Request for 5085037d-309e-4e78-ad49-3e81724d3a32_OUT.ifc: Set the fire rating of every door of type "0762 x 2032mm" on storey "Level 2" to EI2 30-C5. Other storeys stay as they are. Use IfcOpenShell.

First a look at what the model holds.

```python
import ifcopenshell
import ifcopenshell.util.element

model = ifcopenshell.open("5085037d-309e-4e78-ad49-3e81724d3a32_OUT.ifc")
print(model.schema)
storey = next(s for s in model.by_type("IfcBuildingStorey") if s.Name == "Level 2")
doors = [e for e in ifcopenshell.util.element.get_decomposition(storey) if e.is_a("IfcDoor")]
seen = {}
for e in doors:
    element_type = ifcopenshell.util.element.get_type(e)
    key = (element_type.Name if element_type != e and element_type else None, ifcopenshell.util.element.get_pset(e, "Pset_DoorCommon", "FireRating"))
    seen[key] = seen.get(key, 0) + 1
for (name, value), count in sorted(seen.items(), key=str):
    print(count, "x", name, "|", value)
```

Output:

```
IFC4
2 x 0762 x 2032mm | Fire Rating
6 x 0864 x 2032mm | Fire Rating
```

```python
import ifcopenshell
import ifcopenshell.api.pset
import ifcopenshell.util.element

model = ifcopenshell.open("5085037d-309e-4e78-ad49-3e81724d3a32_OUT.ifc")

storey = next(s for s in model.by_type("IfcBuildingStorey") if s.Name == "Level 2")
doors = [e for e in ifcopenshell.util.element.get_decomposition(storey) if e.is_a("IfcDoor")]

count = 0
for e in doors:
    element_type = ifcopenshell.util.element.get_type(e)
    if element_type in (None, e) or element_type.Name != "0762 x 2032mm":
        continue
    # add_pset returns the element's existing set when there is one.
    pset = ifcopenshell.api.pset.add_pset(model, product=e, name="Pset_DoorCommon")
    ifcopenshell.api.pset.edit_pset(model, pset=pset, properties={"FireRating": "EI2 30-C5"})
    count += 1

print(count, "doors updated")

model.write("5085037d-309e-4e78-ad49-3e81724d3a32_OUT-out.ifc")
```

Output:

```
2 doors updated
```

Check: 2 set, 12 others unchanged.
